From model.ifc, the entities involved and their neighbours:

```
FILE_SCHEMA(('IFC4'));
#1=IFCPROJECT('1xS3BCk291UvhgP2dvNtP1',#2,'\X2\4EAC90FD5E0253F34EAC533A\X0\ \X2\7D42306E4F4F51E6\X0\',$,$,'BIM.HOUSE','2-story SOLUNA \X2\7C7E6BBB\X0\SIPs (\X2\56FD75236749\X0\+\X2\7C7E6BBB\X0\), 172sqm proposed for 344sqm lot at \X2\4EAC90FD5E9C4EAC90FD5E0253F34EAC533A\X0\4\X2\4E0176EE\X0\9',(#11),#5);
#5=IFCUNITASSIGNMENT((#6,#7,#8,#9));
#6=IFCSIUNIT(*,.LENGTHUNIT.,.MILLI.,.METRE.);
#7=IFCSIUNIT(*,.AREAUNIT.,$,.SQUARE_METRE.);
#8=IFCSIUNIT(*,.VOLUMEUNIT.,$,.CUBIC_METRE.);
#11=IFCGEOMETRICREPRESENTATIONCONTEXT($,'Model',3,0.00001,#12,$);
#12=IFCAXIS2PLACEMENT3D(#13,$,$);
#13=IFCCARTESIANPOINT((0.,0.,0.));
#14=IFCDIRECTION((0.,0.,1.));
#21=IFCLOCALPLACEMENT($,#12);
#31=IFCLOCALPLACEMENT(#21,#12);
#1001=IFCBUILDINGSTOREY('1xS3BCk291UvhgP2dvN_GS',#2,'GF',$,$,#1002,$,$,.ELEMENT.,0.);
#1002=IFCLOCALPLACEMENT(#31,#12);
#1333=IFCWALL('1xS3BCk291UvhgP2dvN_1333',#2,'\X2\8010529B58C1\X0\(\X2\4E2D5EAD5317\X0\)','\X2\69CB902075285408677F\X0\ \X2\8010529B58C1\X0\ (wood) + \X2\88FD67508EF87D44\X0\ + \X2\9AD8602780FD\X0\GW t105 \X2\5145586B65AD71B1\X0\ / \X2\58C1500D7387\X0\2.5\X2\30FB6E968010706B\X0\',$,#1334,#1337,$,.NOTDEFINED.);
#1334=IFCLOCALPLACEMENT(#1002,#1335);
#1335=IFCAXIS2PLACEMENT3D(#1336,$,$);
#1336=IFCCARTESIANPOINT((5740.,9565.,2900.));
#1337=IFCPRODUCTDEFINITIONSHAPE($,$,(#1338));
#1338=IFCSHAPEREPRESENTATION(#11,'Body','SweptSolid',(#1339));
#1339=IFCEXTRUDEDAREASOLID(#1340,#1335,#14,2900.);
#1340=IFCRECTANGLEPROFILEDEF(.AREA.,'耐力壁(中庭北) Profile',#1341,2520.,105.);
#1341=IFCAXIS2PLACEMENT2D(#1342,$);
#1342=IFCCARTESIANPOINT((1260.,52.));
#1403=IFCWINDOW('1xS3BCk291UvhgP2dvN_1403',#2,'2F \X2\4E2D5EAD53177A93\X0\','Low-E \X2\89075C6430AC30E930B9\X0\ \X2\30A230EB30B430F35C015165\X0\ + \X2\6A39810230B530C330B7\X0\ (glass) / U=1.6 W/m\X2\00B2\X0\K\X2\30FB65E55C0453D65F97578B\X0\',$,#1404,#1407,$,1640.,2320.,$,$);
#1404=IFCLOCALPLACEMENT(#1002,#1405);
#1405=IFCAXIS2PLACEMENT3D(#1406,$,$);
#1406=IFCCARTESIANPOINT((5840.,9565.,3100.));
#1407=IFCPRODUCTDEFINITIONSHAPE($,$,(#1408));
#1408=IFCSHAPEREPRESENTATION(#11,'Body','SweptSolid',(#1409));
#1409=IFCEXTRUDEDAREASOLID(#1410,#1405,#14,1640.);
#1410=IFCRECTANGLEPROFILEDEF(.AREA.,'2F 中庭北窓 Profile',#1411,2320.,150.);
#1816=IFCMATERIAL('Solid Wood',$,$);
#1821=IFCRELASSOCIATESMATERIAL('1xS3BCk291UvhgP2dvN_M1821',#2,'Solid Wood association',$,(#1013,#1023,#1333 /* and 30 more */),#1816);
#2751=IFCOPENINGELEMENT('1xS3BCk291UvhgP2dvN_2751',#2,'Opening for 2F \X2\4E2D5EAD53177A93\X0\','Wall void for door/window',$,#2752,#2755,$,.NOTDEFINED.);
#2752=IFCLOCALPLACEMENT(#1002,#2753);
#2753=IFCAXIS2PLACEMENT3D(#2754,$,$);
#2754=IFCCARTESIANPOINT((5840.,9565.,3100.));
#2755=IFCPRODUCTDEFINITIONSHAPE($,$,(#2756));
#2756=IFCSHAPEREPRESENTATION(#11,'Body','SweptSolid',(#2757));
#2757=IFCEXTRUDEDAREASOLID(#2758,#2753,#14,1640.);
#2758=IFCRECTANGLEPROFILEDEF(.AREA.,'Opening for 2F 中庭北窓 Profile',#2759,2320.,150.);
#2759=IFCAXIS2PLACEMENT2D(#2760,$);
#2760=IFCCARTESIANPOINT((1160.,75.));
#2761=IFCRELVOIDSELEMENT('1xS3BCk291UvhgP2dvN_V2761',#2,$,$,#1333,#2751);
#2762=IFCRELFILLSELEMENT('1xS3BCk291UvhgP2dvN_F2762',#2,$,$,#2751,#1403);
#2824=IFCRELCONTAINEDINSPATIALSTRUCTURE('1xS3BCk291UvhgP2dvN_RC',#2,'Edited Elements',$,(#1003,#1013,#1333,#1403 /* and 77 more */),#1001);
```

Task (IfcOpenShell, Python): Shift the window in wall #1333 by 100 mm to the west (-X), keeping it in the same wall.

```python
import ifcopenshell
import ifcopenshell.api.geometry
import ifcopenshell.util.placement
import ifcopenshell.util.unit

model = ifcopenshell.open("model.ifc")
unit_scale = ifcopenshell.util.unit.calculate_unit_scale(model)

window = model.by_guid("1xS3BCk291UvhgP2dvN_1403")
opening = window.FillsVoids[0].RelatingOpeningElement
wall = opening.VoidsElements[0].RelatingBuildingElement

wall_matrix = ifcopenshell.util.placement.get_local_placement(wall.ObjectPlacement)
shift = wall_matrix[:3, 0] * -0.1 / unit_scale
before = ifcopenshell.util.placement.get_local_placement(window.ObjectPlacement)[:3, 3].copy()

# The window is not placed relative to its opening, so move both.
for product in (opening, window):
    matrix = ifcopenshell.util.placement.get_local_placement(product.ObjectPlacement)
    matrix[:3, 3] += shift
    ifcopenshell.api.geometry.edit_object_placement(model, product=product, matrix=matrix, is_si=False)

after = ifcopenshell.util.placement.get_local_placement(window.ObjectPlacement)[:3, 3]
print("window moved by", (after - before).round(3) + 0.0)

model.write("model_rev.ifc")
```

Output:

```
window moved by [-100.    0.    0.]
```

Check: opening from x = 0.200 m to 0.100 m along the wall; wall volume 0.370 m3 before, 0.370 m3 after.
